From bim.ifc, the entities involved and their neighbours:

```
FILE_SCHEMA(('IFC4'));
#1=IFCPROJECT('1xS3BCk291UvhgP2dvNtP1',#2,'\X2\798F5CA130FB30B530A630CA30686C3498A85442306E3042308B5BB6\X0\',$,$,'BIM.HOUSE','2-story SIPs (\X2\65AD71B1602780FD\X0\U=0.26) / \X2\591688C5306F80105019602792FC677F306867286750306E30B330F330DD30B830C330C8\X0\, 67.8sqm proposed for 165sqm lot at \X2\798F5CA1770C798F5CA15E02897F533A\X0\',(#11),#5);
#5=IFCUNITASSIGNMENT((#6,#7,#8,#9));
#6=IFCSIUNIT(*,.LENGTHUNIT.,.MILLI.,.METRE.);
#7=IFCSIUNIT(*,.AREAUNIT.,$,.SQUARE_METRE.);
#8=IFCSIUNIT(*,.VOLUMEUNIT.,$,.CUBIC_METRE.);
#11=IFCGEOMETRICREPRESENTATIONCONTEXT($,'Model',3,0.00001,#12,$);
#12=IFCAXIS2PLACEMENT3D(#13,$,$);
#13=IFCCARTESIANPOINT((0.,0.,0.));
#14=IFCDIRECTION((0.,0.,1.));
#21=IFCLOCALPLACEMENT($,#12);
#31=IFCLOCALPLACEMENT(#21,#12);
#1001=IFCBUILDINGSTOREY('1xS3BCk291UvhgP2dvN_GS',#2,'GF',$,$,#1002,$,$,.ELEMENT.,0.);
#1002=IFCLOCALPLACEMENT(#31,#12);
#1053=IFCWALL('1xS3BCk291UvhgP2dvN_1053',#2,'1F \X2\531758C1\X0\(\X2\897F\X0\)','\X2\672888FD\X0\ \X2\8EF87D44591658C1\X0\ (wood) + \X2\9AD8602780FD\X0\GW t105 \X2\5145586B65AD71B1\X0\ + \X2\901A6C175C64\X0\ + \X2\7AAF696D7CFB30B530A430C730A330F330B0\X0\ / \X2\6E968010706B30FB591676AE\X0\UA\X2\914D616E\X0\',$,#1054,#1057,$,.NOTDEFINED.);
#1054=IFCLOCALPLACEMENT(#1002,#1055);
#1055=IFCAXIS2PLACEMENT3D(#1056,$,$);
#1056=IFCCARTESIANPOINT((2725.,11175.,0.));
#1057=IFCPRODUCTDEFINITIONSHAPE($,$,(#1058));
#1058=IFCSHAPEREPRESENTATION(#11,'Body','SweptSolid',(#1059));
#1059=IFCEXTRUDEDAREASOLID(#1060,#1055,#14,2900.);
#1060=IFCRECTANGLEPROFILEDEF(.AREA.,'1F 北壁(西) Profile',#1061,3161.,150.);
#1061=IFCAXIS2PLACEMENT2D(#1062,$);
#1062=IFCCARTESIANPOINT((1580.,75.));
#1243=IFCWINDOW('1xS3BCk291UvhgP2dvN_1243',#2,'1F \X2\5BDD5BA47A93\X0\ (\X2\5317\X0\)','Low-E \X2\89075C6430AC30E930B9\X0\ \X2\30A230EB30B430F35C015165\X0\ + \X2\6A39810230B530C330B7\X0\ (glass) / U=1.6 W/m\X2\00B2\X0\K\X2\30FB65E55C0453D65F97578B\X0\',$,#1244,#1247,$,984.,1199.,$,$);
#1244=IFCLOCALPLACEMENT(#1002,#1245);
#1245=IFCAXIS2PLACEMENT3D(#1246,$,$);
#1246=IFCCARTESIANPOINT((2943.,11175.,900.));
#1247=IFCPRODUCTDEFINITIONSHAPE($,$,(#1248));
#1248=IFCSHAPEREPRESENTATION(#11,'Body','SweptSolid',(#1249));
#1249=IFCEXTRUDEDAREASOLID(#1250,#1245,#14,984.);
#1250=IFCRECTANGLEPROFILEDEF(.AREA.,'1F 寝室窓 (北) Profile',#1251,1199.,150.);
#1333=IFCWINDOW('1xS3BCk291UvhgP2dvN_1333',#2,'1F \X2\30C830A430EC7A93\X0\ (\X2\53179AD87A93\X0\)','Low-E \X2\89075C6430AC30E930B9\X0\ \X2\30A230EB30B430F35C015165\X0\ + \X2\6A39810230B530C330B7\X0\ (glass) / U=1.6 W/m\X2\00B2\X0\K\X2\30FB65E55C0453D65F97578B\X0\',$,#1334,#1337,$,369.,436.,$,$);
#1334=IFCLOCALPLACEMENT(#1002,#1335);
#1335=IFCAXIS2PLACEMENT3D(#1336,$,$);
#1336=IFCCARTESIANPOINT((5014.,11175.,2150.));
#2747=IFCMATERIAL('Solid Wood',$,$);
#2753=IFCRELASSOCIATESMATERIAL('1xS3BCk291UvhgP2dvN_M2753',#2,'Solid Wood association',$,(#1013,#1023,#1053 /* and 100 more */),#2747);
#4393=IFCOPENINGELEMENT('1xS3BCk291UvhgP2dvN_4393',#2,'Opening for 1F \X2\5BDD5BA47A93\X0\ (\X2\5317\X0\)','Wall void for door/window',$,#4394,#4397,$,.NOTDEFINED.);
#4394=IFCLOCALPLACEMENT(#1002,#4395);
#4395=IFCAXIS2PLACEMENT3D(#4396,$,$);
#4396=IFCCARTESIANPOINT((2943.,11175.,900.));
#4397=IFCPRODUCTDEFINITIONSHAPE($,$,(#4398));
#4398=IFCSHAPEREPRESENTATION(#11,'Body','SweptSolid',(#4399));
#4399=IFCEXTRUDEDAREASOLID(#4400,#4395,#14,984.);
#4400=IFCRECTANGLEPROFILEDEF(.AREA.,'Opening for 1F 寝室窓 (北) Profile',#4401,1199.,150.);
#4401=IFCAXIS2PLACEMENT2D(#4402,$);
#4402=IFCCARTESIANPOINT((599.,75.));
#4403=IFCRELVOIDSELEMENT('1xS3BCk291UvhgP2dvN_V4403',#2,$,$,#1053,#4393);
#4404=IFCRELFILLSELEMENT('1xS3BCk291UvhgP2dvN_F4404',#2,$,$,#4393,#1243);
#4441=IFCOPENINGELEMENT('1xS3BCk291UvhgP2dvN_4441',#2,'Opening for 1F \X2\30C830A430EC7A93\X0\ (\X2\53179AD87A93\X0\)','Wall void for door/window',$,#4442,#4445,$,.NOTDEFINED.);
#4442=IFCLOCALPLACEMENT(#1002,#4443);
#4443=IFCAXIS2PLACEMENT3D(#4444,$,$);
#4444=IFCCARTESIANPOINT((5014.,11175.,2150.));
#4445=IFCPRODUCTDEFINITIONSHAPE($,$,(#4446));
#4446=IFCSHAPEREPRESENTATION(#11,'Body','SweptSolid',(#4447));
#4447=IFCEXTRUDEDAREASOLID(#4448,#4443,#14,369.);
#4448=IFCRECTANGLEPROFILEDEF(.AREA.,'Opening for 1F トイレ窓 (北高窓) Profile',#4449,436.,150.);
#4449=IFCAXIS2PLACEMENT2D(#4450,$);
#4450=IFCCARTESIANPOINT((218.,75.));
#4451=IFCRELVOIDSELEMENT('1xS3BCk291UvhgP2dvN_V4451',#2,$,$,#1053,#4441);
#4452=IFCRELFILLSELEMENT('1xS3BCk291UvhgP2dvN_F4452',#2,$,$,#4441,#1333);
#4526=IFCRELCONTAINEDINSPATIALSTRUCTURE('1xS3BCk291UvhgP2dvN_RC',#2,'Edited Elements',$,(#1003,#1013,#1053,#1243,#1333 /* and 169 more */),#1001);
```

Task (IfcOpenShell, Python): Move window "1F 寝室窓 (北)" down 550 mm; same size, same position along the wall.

```python
import numpy as np
import ifcopenshell
import ifcopenshell.api.geometry
import ifcopenshell.util.placement
import ifcopenshell.util.unit

model = ifcopenshell.open("bim.ifc")
unit_scale = ifcopenshell.util.unit.calculate_unit_scale(model)

window = model.by_guid("1xS3BCk291UvhgP2dvN_1243")
opening = window.FillsVoids[0].RelatingOpeningElement
dz = -550.0

shift = np.array([0.0, 0.0, dz])
# The window is not placed relative to its opening, so move both.
for product in (opening, window):
    matrix = ifcopenshell.util.placement.get_local_placement(product.ObjectPlacement)
    matrix[:3, 3] += shift
    ifcopenshell.api.geometry.edit_object_placement(model, product=product, matrix=matrix, is_si=False)

print(f"moved by {dz * unit_scale:+.3f} m")

model.write("bim_v2.ifc")
```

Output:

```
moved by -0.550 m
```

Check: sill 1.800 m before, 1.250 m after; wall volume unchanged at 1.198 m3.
